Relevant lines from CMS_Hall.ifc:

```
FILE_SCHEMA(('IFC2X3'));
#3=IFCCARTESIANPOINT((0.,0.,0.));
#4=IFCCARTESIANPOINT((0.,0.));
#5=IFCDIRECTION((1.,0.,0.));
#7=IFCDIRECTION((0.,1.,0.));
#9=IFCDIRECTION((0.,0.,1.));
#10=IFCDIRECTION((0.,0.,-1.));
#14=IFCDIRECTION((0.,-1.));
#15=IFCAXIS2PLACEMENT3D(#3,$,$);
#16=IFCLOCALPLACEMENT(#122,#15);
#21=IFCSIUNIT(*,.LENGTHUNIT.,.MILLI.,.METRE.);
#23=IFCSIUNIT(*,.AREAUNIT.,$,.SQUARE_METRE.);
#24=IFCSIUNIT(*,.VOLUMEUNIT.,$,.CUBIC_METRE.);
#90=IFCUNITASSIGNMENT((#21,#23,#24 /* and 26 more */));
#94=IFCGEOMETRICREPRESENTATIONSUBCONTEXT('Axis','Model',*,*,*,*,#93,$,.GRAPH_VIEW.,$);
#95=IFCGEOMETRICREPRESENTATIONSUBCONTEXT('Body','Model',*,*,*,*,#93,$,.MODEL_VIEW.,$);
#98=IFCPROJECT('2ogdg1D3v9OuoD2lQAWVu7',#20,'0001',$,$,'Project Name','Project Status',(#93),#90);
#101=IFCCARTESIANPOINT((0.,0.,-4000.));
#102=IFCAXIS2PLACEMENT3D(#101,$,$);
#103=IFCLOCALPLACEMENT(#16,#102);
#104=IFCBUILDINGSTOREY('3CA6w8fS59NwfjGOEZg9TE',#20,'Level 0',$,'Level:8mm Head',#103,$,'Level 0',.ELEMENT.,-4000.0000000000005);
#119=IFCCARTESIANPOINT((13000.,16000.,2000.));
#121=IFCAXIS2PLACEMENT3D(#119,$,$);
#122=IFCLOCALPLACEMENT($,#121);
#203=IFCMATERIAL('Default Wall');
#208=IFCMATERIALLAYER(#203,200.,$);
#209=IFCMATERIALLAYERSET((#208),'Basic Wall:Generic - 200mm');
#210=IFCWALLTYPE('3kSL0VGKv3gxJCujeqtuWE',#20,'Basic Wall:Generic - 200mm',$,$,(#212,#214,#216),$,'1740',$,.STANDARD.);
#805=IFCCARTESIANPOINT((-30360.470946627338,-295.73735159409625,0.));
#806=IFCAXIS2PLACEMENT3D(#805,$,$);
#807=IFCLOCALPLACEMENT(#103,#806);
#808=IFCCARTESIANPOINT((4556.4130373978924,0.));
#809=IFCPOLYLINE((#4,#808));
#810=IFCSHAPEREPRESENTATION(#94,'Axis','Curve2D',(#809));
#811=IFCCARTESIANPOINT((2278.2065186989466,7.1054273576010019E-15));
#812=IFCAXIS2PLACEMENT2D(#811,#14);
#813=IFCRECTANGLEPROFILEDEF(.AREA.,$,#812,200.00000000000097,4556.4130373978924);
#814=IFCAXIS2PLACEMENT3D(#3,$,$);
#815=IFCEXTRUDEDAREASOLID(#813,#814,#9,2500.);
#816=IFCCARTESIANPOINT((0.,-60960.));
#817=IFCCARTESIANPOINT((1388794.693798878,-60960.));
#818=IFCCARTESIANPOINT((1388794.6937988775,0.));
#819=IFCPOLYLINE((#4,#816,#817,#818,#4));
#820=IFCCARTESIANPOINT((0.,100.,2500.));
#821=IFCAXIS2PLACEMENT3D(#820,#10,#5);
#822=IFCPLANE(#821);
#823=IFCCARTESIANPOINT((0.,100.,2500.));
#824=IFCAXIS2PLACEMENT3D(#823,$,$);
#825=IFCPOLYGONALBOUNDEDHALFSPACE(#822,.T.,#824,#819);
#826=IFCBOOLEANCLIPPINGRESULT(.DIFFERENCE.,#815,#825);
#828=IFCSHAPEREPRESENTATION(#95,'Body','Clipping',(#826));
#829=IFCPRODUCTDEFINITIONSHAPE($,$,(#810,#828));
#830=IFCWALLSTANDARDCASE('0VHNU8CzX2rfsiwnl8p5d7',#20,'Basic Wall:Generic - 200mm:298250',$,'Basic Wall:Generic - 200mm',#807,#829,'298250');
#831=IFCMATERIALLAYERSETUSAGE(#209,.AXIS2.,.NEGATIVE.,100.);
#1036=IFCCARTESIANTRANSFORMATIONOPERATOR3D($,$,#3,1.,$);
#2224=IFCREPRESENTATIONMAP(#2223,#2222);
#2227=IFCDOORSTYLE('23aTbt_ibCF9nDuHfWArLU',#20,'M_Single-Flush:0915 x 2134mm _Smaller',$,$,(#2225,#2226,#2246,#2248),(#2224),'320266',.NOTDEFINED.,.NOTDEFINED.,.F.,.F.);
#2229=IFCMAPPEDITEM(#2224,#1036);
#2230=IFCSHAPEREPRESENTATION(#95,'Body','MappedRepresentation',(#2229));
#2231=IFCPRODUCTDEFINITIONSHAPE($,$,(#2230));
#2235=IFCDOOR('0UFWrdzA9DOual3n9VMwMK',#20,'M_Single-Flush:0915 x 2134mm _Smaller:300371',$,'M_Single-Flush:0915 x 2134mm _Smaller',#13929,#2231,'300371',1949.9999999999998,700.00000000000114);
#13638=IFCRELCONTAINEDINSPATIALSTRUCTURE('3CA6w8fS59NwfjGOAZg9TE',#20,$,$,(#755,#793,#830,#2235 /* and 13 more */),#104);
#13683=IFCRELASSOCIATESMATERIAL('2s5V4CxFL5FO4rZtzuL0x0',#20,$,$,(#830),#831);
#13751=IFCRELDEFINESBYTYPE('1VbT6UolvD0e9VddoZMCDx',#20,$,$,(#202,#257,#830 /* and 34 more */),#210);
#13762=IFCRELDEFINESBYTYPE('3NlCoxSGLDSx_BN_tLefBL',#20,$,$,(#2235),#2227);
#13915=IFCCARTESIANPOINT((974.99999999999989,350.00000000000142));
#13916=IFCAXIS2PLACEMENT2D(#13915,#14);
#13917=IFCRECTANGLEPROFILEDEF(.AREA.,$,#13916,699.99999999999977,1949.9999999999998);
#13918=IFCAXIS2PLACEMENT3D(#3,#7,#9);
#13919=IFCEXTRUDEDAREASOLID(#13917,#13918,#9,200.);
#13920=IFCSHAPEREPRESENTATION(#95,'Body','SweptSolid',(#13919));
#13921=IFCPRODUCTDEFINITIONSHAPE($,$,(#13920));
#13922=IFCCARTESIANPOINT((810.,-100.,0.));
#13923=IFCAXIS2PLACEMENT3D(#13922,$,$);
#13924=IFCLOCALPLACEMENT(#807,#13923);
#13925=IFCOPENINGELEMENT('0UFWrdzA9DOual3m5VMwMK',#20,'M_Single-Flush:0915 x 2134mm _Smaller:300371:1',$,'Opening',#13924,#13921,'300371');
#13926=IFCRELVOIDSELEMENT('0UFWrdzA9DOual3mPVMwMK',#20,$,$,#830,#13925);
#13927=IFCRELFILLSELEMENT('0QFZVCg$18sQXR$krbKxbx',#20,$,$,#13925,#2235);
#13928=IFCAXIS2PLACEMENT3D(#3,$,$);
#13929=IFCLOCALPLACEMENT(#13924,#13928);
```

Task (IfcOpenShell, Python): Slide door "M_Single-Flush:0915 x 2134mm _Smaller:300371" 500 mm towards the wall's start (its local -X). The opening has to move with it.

```python
import ifcopenshell
import ifcopenshell.api.geometry
import ifcopenshell.util.placement
import ifcopenshell.util.unit

model = ifcopenshell.open("CMS_Hall.ifc")
unit_scale = ifcopenshell.util.unit.calculate_unit_scale(model)

door = model.by_id(2235)
opening = door.FillsVoids[0].RelatingOpeningElement
wall = opening.VoidsElements[0].RelatingBuildingElement

wall_matrix = ifcopenshell.util.placement.get_local_placement(wall.ObjectPlacement)
shift = wall_matrix[:3, 0] * -0.5 / unit_scale
before = ifcopenshell.util.placement.get_local_placement(door.ObjectPlacement)[:3, 3].copy()

# The door is placed relative to its opening, so it follows when the opening moves.
matrix = ifcopenshell.util.placement.get_local_placement(opening.ObjectPlacement)
matrix[:3, 3] += shift
ifcopenshell.api.geometry.edit_object_placement(
    model, product=opening, matrix=matrix, is_si=False, should_transform_children=True
)

after = ifcopenshell.util.placement.get_local_placement(door.ObjectPlacement)[:3, 3]
print("door moved by", (after - before).round(3) + 0.0)

model.write("CMS_Hall_updated.ifc")
```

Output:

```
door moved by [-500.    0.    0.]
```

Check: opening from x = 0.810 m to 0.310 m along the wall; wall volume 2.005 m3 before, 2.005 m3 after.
